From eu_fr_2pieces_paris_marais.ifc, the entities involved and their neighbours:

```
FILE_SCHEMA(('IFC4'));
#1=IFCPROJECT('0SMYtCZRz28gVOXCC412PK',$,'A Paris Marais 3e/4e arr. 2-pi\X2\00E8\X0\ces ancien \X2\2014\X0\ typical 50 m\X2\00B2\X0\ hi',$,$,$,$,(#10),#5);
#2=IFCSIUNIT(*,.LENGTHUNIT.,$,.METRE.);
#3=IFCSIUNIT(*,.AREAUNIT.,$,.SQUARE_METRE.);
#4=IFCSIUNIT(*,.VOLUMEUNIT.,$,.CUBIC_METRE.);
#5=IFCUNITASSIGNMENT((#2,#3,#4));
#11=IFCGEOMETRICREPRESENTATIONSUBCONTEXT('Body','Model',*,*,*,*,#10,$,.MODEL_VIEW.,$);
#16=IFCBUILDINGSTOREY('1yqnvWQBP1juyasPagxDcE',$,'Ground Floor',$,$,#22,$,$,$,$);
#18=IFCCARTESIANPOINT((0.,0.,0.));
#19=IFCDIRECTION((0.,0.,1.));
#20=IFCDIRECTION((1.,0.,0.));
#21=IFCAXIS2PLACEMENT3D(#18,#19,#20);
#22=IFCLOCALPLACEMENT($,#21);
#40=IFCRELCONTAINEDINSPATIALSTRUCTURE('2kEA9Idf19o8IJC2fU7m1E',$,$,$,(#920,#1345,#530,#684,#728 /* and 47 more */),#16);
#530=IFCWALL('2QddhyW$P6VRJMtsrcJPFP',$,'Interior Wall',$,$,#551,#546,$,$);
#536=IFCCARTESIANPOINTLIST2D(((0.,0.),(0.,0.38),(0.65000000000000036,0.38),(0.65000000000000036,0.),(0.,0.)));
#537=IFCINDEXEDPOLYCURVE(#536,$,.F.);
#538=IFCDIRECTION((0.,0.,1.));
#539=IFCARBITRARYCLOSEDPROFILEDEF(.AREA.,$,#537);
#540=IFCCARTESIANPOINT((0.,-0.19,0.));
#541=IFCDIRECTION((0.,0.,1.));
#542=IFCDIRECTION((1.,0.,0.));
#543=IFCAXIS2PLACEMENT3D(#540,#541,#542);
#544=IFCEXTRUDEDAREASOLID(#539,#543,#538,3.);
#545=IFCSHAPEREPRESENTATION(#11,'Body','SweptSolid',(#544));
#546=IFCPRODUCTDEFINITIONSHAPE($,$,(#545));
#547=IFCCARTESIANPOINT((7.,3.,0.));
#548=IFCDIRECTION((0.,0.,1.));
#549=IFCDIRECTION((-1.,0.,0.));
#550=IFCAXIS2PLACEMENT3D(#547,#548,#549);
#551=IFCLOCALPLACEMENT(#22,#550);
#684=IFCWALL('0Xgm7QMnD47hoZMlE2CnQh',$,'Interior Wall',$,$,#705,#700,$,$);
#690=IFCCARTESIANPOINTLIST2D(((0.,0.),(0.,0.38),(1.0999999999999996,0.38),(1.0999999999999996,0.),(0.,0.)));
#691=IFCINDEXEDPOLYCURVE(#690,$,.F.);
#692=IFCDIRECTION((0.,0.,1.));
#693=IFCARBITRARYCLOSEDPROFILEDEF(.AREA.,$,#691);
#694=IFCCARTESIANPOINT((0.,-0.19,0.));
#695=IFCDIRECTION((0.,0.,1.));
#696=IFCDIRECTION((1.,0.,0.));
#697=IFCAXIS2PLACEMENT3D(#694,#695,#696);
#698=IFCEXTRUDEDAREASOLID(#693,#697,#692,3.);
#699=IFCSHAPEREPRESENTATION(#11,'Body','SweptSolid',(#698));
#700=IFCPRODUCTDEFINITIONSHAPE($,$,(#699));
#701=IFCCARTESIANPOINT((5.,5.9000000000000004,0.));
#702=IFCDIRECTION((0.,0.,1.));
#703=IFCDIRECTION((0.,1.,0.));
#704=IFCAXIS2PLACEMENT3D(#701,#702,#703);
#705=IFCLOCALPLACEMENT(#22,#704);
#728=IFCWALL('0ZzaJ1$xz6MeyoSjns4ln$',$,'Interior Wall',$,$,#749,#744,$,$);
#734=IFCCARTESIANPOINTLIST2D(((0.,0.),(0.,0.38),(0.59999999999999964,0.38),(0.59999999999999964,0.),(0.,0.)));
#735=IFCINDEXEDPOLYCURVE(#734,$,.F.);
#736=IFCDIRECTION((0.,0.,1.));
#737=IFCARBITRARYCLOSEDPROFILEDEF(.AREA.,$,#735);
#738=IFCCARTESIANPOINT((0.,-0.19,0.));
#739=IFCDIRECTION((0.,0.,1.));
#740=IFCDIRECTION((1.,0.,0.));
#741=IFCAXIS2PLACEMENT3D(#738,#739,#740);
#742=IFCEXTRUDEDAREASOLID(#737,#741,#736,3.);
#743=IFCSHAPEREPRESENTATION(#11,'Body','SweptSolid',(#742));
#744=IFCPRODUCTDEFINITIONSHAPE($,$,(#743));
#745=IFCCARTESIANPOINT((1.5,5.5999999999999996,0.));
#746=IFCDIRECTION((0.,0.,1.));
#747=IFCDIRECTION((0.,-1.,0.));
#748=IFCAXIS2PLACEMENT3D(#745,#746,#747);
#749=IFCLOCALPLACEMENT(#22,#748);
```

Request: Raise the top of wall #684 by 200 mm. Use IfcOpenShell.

```python
import ifcopenshell
import ifcopenshell.geom
import ifcopenshell.util.representation
import ifcopenshell.util.shape
import ifcopenshell.util.unit

model = ifcopenshell.open("eu_fr_2pieces_paris_marais.ifc")
unit_scale = ifcopenshell.util.unit.calculate_unit_scale(model)
settings = ifcopenshell.geom.settings()


def volume(element):
    """Net volume in cubic metres, openings subtracted."""
    shape = ifcopenshell.geom.create_shape(settings, element)
    return ifcopenshell.util.shape.get_volume(shape.geometry)


wall = model.by_id(684)
before = volume(wall)

body = ifcopenshell.util.representation.get_representation(wall, "Model", "Body")
solid = body.Items[0]
old_height = solid.Depth
solid.Depth += 0.2 / unit_scale
after = volume(wall)

print(f"height {old_height:g} -> {solid.Depth:g}, volume {before:.3f} -> {after:.3f} m3")

model.write("eu_fr_2pieces_paris_marais_rev.ifc")
```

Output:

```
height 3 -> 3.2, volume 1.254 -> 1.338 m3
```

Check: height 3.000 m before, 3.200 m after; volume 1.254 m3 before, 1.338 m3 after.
